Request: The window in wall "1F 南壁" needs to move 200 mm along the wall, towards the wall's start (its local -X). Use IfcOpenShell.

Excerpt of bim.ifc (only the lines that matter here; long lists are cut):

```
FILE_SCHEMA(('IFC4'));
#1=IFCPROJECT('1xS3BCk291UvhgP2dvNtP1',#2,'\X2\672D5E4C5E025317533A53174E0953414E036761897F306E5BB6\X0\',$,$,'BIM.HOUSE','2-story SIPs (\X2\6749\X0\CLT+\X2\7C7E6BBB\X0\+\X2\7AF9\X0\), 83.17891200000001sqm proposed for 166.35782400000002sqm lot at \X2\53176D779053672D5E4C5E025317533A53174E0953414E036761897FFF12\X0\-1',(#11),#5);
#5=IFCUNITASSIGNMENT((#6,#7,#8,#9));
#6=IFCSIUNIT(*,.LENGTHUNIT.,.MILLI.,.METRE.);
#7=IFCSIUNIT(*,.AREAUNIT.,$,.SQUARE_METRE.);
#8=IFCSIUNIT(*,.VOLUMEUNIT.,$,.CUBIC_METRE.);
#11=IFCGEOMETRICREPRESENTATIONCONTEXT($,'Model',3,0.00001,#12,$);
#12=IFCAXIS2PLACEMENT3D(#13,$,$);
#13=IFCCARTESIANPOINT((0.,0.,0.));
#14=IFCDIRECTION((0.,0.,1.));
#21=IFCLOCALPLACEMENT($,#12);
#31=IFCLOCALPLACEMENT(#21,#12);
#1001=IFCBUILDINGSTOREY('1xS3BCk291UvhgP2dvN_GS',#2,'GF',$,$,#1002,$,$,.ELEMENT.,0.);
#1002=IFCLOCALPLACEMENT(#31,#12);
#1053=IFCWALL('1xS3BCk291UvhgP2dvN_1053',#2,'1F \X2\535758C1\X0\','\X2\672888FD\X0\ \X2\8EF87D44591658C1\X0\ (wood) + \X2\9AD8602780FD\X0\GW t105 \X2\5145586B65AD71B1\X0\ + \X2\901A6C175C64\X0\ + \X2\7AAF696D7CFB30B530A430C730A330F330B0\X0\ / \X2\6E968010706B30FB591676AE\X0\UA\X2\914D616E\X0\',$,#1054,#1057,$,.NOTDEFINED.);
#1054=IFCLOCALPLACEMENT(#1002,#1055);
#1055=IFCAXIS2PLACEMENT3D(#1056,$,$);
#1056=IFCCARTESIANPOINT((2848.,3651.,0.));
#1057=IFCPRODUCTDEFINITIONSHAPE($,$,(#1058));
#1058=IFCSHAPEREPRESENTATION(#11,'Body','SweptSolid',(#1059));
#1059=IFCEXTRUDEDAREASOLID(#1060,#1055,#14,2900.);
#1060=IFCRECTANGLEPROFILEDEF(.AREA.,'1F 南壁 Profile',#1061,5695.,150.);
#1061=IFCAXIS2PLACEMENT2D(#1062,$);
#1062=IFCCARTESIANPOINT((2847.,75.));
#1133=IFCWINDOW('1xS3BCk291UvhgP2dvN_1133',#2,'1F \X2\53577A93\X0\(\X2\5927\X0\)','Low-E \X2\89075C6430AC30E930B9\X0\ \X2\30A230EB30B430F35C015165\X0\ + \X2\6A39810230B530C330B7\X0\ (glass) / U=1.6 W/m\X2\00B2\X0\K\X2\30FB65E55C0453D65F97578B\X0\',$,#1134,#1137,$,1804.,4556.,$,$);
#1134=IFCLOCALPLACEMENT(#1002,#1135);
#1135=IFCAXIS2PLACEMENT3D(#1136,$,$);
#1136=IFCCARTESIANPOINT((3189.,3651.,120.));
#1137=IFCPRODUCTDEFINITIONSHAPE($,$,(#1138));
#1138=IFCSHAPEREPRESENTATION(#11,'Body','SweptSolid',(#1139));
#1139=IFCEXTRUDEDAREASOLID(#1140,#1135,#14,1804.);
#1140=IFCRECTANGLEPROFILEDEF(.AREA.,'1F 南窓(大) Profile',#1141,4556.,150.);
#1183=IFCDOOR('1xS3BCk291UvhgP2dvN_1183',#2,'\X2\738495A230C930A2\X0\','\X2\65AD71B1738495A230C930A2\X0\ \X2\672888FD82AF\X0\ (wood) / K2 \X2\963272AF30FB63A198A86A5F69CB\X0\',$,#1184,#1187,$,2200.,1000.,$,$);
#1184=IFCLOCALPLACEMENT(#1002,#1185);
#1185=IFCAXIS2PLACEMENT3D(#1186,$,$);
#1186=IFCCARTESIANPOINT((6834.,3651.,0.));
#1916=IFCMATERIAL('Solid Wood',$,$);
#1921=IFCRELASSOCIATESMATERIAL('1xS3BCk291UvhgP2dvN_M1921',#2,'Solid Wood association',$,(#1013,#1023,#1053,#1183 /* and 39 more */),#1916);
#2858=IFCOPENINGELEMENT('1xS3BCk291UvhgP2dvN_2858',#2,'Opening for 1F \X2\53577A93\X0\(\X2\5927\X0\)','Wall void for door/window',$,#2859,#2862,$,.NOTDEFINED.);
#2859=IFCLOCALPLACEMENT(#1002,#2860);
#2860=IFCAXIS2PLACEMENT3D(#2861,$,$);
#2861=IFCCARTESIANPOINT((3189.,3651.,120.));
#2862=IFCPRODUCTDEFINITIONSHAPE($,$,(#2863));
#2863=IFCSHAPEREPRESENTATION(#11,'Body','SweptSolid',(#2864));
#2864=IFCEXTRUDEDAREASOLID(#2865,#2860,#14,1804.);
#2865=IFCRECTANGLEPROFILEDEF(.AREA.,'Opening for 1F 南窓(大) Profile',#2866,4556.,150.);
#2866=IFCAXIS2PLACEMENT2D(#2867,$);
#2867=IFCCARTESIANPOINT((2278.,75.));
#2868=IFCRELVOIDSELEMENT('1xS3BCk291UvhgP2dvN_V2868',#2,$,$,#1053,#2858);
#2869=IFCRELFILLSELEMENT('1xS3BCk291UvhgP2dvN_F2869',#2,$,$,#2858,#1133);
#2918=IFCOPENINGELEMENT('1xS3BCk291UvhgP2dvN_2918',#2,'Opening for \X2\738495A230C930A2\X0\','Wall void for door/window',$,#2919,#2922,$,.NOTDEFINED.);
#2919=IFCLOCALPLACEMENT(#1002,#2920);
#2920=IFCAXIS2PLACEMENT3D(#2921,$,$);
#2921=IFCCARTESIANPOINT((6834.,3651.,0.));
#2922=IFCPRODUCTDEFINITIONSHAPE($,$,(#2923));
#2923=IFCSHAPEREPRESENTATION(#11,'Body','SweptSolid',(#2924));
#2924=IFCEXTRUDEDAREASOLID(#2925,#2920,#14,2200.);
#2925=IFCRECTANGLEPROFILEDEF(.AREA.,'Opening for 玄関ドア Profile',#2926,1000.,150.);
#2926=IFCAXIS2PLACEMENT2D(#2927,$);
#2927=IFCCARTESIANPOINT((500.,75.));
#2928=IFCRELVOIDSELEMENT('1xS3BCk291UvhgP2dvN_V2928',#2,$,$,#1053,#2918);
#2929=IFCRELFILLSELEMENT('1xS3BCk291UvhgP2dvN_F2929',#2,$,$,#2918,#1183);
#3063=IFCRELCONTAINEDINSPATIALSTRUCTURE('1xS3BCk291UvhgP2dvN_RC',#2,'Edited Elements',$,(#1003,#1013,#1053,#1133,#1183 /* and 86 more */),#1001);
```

```python
import ifcopenshell
import ifcopenshell.api.geometry
import ifcopenshell.util.placement

model = ifcopenshell.open("bim.ifc")

window = model.by_id(1133)
opening = window.FillsVoids[0].RelatingOpeningElement
wall = opening.VoidsElements[0].RelatingBuildingElement

wall_matrix = ifcopenshell.util.placement.get_local_placement(wall.ObjectPlacement)
shift = wall_matrix[:3, 0] * -200.0
before = ifcopenshell.util.placement.get_local_placement(window.ObjectPlacement)[:3, 3].copy()

# The window is not placed relative to its opening, so move both.
for product in (opening, window):
    matrix = ifcopenshell.util.placement.get_local_placement(product.ObjectPlacement)
    matrix[:3, 3] += shift
    ifcopenshell.api.geometry.edit_object_placement(model, product=product, matrix=matrix, is_si=False)

after = ifcopenshell.util.placement.get_local_placement(window.ObjectPlacement)[:3, 3]
print("window moved by", (after - before).round(3) + 0.0)

model.write("bim_v2.ifc")
```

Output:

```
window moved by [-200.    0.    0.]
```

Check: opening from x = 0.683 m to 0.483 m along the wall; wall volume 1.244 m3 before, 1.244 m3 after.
